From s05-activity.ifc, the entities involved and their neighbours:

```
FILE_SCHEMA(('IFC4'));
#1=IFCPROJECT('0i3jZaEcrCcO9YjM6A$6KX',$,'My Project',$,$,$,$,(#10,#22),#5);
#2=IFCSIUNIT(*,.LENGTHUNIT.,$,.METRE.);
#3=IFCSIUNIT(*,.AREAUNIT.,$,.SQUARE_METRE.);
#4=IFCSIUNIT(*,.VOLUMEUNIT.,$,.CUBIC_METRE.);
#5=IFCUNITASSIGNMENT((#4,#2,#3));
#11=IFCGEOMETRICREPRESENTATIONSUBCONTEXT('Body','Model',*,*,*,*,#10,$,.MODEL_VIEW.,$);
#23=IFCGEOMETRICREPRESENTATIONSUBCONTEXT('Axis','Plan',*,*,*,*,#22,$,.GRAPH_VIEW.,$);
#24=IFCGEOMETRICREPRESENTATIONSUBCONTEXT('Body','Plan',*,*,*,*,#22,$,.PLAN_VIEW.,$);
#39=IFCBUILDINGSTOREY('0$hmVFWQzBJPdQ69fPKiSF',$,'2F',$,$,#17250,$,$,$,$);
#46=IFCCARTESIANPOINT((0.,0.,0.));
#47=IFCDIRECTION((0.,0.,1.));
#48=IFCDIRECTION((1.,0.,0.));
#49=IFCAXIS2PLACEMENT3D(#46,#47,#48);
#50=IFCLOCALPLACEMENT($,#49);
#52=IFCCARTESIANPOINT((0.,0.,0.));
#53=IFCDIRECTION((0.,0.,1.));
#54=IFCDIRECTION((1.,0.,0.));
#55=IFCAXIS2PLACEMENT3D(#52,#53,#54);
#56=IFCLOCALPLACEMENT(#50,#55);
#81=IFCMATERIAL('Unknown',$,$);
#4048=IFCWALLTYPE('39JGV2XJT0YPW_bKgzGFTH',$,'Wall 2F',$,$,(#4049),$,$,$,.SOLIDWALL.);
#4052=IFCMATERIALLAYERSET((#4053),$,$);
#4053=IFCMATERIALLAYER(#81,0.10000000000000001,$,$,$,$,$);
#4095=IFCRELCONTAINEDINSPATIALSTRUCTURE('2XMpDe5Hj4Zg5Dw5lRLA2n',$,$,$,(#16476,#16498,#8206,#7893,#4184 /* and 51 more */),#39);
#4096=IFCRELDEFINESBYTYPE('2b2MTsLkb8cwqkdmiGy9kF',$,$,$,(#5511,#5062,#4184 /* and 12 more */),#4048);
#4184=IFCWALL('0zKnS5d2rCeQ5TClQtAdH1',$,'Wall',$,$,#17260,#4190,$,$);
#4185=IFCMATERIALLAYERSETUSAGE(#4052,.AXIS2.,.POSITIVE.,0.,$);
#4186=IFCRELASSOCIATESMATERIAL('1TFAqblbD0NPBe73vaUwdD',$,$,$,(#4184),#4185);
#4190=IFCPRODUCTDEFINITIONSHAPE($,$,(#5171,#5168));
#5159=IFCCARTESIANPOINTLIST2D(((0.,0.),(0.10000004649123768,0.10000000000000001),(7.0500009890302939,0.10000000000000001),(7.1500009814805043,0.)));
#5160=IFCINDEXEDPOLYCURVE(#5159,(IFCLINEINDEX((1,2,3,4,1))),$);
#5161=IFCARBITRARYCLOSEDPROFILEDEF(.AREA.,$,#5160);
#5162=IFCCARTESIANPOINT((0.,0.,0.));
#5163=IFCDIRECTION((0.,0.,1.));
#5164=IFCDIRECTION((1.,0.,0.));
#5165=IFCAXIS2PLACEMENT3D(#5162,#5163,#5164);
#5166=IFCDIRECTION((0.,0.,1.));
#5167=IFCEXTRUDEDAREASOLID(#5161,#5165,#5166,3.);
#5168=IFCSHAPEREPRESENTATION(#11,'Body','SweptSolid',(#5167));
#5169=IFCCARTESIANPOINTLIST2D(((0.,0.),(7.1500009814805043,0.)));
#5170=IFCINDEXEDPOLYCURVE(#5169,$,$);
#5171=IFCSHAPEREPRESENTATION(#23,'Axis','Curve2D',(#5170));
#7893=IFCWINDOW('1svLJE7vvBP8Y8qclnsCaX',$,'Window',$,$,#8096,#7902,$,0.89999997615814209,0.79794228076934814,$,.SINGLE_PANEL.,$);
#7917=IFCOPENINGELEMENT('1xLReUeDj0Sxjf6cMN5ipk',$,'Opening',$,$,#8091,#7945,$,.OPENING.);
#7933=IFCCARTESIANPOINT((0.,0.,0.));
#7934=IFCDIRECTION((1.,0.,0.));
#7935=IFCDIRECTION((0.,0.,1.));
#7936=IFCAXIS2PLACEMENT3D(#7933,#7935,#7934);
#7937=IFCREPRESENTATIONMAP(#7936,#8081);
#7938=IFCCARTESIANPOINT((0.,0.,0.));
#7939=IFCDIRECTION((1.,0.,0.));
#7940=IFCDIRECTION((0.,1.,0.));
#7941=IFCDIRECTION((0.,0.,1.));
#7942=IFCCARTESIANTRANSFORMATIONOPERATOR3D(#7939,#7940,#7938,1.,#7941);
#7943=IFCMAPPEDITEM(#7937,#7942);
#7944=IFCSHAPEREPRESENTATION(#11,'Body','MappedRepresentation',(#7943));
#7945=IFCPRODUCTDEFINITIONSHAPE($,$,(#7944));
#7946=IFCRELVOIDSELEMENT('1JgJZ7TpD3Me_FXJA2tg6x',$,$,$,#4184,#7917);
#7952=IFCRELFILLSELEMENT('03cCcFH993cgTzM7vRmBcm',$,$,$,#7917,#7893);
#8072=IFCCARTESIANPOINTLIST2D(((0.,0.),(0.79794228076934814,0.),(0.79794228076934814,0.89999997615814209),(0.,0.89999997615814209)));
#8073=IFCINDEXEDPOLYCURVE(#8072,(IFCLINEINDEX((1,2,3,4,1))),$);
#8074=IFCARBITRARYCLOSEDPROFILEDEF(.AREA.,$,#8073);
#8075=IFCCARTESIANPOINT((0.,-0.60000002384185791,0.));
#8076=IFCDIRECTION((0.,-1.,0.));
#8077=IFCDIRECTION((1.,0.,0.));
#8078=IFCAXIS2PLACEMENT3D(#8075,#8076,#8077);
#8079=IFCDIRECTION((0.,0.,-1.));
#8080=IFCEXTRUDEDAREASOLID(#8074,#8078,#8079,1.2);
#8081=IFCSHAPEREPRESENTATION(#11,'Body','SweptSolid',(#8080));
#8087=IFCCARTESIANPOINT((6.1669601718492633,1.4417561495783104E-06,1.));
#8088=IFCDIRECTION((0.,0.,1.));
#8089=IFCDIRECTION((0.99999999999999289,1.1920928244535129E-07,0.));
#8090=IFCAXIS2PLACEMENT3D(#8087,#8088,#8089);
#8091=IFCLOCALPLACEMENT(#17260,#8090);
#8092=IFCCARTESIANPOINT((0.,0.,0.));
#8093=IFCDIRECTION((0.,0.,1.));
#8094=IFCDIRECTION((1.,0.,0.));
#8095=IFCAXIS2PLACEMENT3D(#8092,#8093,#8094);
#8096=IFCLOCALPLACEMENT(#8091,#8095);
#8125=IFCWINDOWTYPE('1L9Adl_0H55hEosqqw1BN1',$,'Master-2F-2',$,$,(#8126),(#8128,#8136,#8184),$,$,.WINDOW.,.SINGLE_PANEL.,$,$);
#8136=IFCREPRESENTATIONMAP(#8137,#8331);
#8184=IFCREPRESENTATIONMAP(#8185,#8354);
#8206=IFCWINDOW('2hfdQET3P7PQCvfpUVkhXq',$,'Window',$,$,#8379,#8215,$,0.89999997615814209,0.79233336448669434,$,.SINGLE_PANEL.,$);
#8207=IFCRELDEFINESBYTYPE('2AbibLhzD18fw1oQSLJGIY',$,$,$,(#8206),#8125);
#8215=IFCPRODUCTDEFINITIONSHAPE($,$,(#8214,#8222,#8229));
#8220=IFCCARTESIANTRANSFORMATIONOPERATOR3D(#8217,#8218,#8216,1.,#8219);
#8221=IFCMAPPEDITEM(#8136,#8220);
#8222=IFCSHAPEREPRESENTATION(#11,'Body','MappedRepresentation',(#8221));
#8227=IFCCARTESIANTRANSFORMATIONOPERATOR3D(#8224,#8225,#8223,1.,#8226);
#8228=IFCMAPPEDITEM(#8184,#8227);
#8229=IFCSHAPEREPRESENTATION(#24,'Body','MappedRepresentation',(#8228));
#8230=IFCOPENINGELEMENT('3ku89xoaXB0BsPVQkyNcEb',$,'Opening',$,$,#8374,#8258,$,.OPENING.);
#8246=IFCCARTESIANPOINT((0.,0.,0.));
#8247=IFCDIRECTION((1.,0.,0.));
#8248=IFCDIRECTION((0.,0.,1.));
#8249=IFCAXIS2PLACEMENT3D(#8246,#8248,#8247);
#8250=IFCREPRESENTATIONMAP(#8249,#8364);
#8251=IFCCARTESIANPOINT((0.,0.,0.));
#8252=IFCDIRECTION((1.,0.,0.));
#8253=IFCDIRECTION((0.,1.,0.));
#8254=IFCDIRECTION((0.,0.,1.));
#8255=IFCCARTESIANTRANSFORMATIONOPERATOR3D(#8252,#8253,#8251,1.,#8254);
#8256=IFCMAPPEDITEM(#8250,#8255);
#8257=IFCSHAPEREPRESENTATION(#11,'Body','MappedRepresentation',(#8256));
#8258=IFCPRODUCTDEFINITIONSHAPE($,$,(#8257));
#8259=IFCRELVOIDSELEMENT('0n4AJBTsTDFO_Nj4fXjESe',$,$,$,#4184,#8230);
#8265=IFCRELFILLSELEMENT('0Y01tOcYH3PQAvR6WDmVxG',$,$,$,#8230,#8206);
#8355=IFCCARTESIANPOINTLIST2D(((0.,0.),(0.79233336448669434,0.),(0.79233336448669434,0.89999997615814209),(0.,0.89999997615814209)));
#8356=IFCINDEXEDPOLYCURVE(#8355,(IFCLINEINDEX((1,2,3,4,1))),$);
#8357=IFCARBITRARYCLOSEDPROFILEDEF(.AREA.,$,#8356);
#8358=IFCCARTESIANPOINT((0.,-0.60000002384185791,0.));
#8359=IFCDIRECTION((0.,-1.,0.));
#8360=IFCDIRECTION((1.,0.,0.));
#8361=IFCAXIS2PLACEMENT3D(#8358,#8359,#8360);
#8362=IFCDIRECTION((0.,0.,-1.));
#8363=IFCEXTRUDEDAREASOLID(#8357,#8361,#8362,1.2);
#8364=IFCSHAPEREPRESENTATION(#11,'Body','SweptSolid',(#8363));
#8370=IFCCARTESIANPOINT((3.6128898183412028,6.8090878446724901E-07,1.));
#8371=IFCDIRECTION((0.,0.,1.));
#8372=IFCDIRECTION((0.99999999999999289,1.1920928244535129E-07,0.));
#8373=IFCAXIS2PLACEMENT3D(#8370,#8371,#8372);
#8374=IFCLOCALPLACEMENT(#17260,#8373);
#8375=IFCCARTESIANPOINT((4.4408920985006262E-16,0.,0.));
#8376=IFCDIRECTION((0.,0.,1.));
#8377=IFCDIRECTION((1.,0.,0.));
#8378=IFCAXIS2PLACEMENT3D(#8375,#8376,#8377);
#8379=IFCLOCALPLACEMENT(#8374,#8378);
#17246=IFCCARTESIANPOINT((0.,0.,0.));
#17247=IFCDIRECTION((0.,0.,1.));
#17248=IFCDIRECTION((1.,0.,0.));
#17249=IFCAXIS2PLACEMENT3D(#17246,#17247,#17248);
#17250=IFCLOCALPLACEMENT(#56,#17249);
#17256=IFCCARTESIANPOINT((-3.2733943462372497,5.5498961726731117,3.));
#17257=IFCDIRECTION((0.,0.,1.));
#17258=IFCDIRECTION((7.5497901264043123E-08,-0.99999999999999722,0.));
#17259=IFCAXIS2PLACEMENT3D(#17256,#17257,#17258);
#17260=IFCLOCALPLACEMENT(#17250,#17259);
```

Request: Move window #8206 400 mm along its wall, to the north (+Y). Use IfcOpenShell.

```python
import ifcopenshell
import ifcopenshell.api.geometry
import ifcopenshell.util.placement

model = ifcopenshell.open("s05-activity.ifc")

window = model.by_guid("2hfdQET3P7PQCvfpUVkhXq")
opening = window.FillsVoids[0].RelatingOpeningElement
wall = opening.VoidsElements[0].RelatingBuildingElement

wall_matrix = ifcopenshell.util.placement.get_local_placement(wall.ObjectPlacement)
shift = wall_matrix[:3, 0] * -0.4
before = ifcopenshell.util.placement.get_local_placement(window.ObjectPlacement)[:3, 3].copy()

# The window is placed relative to its opening, so it follows when the opening moves.
matrix = ifcopenshell.util.placement.get_local_placement(opening.ObjectPlacement)
matrix[:3, 3] += shift
ifcopenshell.api.geometry.edit_object_placement(
    model, product=opening, matrix=matrix, is_si=False, should_transform_children=True
)

after = ifcopenshell.util.placement.get_local_placement(window.ObjectPlacement)[:3, 3]
print("window moved by", (after - before).round(3) + 0.0)

model.write("s05-activity_updated.ifc")
```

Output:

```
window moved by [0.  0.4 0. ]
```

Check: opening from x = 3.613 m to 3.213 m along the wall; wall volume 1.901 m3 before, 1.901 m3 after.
